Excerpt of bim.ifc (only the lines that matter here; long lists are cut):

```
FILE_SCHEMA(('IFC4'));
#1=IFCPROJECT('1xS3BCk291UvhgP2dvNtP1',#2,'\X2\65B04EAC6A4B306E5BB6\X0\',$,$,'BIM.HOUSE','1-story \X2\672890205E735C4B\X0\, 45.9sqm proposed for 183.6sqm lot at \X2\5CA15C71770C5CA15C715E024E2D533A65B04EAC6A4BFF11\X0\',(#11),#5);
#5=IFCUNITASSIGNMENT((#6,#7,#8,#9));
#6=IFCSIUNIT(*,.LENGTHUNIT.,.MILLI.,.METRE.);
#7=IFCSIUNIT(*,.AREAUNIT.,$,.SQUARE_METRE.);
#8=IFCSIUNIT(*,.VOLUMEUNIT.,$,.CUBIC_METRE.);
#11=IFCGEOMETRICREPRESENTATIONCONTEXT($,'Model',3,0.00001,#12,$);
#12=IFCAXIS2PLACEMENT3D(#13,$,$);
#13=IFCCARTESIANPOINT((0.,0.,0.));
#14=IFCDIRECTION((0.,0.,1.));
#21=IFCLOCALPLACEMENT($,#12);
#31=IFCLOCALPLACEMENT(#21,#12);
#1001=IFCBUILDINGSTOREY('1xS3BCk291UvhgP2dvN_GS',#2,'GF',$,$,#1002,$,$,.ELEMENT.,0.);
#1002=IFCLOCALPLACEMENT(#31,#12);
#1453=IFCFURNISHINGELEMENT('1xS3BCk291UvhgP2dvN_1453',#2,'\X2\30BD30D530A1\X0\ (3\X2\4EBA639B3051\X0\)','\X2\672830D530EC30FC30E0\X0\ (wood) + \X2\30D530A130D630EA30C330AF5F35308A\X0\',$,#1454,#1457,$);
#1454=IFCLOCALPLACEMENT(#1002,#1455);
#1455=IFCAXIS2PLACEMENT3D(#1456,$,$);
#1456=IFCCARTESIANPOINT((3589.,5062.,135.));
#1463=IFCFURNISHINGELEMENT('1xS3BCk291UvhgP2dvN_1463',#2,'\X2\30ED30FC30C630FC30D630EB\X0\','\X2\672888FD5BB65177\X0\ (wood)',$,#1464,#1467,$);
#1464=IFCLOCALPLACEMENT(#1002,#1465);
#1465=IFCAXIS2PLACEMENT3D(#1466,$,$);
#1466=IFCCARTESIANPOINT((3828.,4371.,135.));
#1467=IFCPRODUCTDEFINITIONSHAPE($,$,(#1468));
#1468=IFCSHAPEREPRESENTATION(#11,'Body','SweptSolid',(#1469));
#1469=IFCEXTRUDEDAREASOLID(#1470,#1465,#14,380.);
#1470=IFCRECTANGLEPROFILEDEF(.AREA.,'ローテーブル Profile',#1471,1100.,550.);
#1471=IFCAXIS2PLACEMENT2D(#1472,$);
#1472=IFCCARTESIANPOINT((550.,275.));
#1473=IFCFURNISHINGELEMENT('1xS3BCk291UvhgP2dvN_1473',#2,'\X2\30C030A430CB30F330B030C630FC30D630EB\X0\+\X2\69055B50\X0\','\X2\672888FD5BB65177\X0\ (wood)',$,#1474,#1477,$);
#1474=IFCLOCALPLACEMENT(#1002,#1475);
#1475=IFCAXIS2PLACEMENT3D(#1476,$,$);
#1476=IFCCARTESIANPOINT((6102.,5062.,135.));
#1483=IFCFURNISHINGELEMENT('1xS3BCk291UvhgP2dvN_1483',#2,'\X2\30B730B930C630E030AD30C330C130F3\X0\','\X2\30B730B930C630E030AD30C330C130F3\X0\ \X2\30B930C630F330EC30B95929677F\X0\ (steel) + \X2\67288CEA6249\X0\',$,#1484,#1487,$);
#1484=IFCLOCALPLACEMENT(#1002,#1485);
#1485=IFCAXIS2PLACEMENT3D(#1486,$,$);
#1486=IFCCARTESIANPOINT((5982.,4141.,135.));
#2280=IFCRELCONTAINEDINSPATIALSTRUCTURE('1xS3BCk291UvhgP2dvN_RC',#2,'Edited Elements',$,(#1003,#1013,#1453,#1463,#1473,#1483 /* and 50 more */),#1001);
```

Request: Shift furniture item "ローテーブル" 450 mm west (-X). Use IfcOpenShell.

```python
import ifcopenshell
import ifcopenshell.api.geometry
import ifcopenshell.util.placement

model = ifcopenshell.open("bim.ifc")

item = model.by_guid("1xS3BCk291UvhgP2dvN_1463")
matrix = ifcopenshell.util.placement.get_local_placement(item.ObjectPlacement)
matrix[0, 3] -= 450.0
ifcopenshell.api.geometry.edit_object_placement(model, product=item, matrix=matrix, is_si=False)

print(ifcopenshell.util.placement.get_local_placement(item.ObjectPlacement).round(3) + 0.0)

model.write("bim_updated.ifc")
```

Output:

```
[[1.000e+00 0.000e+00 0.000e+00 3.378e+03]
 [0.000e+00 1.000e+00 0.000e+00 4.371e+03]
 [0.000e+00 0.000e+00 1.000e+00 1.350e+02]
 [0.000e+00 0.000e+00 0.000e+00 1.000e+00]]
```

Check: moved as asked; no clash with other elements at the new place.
